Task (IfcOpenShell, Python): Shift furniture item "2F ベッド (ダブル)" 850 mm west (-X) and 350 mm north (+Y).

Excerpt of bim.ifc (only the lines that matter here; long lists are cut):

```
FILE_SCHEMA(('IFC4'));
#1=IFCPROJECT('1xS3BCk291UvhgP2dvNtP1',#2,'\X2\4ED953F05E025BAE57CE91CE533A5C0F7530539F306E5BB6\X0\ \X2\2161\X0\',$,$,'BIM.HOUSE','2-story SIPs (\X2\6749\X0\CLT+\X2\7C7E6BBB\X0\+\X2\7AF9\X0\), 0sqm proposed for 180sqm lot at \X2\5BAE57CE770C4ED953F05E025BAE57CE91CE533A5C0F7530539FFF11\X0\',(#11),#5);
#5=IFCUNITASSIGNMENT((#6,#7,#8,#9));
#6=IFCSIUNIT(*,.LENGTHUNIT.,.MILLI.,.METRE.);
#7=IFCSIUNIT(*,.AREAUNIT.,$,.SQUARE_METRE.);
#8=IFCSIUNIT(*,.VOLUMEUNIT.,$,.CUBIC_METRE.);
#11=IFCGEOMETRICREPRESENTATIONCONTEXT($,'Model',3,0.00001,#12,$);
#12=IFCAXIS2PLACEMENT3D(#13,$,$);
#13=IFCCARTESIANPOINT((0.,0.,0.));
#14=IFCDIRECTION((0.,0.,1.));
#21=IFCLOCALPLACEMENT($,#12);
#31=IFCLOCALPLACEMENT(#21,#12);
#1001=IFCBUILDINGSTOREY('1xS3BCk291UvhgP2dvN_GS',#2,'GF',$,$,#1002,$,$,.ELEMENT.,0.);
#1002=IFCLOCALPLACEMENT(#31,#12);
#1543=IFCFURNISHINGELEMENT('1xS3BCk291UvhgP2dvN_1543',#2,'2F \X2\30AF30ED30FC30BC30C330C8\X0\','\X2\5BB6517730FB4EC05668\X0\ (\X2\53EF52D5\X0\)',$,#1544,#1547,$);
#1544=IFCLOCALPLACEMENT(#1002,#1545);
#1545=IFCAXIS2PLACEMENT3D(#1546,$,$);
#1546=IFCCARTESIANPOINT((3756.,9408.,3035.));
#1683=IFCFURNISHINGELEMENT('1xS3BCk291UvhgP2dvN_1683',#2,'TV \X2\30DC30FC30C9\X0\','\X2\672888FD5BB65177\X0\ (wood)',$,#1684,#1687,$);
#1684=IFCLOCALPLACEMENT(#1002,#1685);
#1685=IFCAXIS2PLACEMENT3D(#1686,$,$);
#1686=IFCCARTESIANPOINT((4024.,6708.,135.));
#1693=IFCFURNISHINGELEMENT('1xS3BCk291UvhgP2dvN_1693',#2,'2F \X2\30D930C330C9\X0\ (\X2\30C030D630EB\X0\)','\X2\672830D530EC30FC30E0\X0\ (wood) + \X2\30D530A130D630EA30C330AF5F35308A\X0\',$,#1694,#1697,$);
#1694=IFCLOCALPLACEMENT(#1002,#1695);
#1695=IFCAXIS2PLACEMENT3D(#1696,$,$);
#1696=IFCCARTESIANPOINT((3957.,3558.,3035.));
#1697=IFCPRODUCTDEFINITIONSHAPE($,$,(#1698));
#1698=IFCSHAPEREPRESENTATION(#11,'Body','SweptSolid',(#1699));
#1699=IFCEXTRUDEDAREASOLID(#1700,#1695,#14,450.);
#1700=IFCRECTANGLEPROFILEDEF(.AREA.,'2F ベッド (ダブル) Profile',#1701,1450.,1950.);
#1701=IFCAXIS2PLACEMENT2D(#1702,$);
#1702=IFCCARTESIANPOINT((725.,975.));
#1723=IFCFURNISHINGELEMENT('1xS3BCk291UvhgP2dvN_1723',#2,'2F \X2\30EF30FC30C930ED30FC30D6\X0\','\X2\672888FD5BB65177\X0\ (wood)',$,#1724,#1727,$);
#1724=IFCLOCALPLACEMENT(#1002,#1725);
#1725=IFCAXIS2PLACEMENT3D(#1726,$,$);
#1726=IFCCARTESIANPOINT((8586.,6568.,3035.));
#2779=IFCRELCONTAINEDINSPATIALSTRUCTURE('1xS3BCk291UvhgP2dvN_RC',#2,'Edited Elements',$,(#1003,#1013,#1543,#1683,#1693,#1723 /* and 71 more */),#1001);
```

```python
import ifcopenshell
import ifcopenshell.api.geometry
import ifcopenshell.util.placement

model = ifcopenshell.open("bim.ifc")

item = model.by_guid("1xS3BCk291UvhgP2dvN_1693")
matrix = ifcopenshell.util.placement.get_local_placement(item.ObjectPlacement)
matrix[0, 3] -= 850.0
matrix[1, 3] += 350.0
ifcopenshell.api.geometry.edit_object_placement(model, product=item, matrix=matrix, is_si=False)

print(ifcopenshell.util.placement.get_local_placement(item.ObjectPlacement).round(3) + 0.0)

model.write("bim_edited.ifc")
```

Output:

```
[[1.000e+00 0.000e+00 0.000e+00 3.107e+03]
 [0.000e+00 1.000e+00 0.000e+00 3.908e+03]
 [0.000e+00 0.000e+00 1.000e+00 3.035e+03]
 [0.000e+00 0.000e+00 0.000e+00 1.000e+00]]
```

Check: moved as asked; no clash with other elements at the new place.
